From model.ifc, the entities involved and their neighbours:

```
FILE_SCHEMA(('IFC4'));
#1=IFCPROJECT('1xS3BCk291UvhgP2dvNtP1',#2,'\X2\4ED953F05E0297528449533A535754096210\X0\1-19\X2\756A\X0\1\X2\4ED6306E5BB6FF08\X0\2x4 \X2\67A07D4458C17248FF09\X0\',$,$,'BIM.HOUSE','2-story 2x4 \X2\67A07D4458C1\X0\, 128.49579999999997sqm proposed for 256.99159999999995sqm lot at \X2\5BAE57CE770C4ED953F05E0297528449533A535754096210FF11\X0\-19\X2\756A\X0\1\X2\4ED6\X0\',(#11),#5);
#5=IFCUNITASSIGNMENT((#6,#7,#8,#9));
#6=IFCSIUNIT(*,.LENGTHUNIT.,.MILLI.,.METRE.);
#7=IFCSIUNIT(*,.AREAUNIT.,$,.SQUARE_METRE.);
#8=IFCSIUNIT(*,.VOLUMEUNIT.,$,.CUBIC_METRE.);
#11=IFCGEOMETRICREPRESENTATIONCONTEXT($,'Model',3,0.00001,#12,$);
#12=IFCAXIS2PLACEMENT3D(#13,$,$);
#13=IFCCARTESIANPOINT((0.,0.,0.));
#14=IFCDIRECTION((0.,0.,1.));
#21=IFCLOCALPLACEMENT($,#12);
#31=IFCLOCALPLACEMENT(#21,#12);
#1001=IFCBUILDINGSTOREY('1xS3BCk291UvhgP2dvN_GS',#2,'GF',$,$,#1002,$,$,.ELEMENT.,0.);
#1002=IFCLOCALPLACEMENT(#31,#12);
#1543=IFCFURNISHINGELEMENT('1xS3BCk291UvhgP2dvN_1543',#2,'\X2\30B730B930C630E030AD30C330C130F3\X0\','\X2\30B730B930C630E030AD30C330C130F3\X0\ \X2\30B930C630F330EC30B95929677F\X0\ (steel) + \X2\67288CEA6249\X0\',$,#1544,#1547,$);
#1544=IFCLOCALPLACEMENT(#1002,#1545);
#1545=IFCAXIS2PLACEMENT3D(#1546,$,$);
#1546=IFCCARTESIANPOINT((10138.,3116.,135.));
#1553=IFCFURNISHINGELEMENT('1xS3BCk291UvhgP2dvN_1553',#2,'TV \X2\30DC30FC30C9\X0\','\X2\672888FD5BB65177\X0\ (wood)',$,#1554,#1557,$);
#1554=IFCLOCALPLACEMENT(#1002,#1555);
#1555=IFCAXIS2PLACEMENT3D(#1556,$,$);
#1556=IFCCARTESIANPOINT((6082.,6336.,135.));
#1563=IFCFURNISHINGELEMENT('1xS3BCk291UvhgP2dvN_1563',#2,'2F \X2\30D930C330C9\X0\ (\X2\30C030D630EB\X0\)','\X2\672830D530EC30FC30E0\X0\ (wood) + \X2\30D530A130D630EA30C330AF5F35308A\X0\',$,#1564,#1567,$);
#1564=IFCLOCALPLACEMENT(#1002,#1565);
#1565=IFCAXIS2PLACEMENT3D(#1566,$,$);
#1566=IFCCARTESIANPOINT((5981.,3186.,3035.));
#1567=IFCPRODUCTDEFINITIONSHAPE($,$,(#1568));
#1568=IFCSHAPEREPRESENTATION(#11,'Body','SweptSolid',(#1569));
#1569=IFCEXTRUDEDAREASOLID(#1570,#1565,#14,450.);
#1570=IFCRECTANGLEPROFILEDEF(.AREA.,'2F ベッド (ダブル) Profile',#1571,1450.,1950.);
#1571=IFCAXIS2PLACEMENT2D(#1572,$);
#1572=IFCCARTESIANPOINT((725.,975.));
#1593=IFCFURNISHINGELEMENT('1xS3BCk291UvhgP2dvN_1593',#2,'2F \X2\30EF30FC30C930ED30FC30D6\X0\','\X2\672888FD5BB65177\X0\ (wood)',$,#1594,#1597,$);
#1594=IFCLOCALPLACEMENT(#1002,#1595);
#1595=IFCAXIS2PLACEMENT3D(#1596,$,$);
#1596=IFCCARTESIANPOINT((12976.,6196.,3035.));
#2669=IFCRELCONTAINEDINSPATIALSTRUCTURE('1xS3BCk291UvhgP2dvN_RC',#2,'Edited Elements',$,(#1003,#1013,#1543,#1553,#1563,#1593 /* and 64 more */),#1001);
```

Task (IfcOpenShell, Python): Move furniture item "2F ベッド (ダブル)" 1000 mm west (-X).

```python
import ifcopenshell
import ifcopenshell.api.geometry
import ifcopenshell.util.placement
import ifcopenshell.util.unit

model = ifcopenshell.open("model.ifc")
unit_scale = ifcopenshell.util.unit.calculate_unit_scale(model)

item = model.by_id(1563)
matrix = ifcopenshell.util.placement.get_local_placement(item.ObjectPlacement)
matrix[0, 3] -= 1 / unit_scale
ifcopenshell.api.geometry.edit_object_placement(model, product=item, matrix=matrix, is_si=False)

print(ifcopenshell.util.placement.get_local_placement(item.ObjectPlacement).round(3) + 0.0)

model.write("model_v2.ifc")
```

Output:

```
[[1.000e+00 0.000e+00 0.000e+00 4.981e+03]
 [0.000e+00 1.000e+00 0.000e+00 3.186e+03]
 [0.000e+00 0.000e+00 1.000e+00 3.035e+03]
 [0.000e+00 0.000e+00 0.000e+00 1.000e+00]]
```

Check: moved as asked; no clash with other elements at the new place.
